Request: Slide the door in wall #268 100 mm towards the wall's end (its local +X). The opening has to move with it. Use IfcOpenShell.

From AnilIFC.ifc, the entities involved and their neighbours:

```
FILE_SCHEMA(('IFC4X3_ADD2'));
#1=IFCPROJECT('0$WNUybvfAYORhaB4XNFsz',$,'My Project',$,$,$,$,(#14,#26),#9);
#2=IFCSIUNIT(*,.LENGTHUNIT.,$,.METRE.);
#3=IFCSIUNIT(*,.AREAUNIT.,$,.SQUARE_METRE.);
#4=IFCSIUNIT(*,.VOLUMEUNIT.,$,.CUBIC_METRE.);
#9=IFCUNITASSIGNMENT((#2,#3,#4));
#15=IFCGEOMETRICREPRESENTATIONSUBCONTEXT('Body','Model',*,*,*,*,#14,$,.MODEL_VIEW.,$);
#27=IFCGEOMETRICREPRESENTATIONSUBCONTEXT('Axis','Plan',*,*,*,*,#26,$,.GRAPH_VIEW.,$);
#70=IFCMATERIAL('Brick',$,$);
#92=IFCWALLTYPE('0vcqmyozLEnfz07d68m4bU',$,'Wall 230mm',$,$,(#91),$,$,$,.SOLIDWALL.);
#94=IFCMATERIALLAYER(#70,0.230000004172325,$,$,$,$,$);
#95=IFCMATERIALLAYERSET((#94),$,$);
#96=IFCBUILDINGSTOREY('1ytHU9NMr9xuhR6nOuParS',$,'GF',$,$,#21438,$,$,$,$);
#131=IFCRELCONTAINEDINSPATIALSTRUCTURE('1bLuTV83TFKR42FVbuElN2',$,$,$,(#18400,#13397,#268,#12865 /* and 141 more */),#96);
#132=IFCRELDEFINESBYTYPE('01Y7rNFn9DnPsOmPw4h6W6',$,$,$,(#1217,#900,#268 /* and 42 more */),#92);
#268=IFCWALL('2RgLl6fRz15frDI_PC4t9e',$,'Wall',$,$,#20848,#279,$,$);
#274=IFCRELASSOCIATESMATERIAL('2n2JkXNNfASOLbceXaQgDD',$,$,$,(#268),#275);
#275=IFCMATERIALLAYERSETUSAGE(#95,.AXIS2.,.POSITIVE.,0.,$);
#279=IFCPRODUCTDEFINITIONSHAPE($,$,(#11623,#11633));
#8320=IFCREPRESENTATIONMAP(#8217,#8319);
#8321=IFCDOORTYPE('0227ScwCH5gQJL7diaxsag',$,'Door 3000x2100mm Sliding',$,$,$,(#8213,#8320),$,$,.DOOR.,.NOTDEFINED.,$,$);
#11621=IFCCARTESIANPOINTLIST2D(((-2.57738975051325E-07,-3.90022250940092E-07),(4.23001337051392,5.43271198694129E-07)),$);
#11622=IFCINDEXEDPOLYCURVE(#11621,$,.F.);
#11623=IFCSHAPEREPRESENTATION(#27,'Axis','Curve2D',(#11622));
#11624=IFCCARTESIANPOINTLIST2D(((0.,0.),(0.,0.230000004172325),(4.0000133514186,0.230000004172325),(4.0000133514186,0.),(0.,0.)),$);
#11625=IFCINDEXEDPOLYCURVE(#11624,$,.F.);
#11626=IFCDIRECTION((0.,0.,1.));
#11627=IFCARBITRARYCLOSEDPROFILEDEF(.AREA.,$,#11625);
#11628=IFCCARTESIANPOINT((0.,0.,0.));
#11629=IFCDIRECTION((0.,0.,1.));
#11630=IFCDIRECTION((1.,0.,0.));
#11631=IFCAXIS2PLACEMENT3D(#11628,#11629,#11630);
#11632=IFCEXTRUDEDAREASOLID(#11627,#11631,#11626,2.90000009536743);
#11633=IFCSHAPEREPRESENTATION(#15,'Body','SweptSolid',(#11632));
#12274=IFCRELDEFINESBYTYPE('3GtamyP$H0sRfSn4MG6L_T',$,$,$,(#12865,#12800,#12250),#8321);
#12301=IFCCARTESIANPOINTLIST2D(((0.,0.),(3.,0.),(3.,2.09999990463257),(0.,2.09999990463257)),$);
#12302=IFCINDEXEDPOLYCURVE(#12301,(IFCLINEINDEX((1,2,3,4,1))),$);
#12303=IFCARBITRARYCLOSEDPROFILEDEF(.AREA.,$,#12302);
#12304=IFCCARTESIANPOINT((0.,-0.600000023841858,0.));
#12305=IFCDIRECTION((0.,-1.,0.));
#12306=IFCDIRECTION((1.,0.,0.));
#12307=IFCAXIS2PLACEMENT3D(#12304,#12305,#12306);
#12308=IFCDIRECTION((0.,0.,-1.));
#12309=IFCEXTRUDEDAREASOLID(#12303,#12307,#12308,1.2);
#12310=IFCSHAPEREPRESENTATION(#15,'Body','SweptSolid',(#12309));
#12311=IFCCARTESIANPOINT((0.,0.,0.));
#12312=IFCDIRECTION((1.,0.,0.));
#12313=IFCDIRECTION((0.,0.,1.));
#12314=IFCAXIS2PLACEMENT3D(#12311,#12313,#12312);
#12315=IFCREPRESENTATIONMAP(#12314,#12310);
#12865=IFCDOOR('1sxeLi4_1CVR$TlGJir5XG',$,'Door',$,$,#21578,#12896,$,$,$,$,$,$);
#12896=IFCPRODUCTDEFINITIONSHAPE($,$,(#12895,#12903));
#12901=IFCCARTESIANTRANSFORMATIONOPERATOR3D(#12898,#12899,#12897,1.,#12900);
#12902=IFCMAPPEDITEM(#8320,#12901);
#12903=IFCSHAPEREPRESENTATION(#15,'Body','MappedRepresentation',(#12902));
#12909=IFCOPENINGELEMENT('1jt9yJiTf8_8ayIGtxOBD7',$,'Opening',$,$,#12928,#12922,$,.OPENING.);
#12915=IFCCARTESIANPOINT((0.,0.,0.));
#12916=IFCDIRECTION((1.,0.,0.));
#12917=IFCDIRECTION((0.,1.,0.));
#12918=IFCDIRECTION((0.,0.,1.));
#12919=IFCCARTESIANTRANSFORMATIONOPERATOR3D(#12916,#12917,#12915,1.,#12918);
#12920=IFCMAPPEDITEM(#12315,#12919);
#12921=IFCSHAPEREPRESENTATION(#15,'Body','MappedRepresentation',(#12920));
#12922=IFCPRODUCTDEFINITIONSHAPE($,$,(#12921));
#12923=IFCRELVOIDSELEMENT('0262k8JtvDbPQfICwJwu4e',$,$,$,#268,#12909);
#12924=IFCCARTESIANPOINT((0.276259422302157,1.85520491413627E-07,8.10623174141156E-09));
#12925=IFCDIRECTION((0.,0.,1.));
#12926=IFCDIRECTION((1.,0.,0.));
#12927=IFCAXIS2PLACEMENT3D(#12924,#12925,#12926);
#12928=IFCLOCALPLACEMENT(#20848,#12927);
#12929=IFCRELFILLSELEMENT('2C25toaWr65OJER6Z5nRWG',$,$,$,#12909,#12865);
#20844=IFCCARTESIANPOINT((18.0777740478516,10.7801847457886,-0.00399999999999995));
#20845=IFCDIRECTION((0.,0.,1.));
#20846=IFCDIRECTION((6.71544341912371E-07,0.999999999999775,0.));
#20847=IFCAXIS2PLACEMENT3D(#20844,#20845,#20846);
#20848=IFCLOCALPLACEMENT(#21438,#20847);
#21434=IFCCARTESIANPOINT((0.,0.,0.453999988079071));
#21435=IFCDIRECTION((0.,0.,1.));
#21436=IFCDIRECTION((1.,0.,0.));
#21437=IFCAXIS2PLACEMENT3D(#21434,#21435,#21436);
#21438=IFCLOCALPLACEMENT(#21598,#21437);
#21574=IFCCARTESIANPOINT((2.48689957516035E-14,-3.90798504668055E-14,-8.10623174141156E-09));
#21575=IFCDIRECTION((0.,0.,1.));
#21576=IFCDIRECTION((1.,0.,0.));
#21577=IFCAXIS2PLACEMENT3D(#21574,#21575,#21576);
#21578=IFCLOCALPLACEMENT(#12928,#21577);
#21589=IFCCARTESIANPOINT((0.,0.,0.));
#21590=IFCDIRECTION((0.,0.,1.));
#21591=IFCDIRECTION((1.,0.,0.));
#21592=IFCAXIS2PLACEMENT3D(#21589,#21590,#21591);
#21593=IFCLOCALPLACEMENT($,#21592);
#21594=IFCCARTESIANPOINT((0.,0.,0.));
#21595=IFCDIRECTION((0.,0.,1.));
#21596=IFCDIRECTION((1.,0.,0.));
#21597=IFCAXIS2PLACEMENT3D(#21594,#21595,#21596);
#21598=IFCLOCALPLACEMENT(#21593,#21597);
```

```python
import ifcopenshell
import ifcopenshell.api.geometry
import ifcopenshell.util.placement

model = ifcopenshell.open("AnilIFC.ifc")

door = model.by_guid("1sxeLi4_1CVR$TlGJir5XG")
opening = door.FillsVoids[0].RelatingOpeningElement
wall = opening.VoidsElements[0].RelatingBuildingElement

wall_matrix = ifcopenshell.util.placement.get_local_placement(wall.ObjectPlacement)
shift = wall_matrix[:3, 0] * 0.1
before = ifcopenshell.util.placement.get_local_placement(door.ObjectPlacement)[:3, 3].copy()

# The door is placed relative to its opening, so it follows when the opening moves.
matrix = ifcopenshell.util.placement.get_local_placement(opening.ObjectPlacement)
matrix[:3, 3] += shift
ifcopenshell.api.geometry.edit_object_placement(
    model, product=opening, matrix=matrix, is_si=False, should_transform_children=True
)

after = ifcopenshell.util.placement.get_local_placement(door.ObjectPlacement)[:3, 3]
print("door moved by", (after - before).round(3) + 0.0)

model.write("AnilIFC-out.ifc")
```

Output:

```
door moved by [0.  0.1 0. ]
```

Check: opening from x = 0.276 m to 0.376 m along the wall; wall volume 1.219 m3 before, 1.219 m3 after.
